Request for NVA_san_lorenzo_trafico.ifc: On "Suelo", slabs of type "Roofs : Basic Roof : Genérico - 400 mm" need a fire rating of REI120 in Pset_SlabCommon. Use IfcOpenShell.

First a look at what the model holds.

```python
import ifcopenshell
import ifcopenshell.util.element

model = ifcopenshell.open("NVA_san_lorenzo_trafico.ifc")
print(model.schema)
storey = next(s for s in model.by_type("IfcBuildingStorey") if s.Name == "Suelo")
slabs = [e for e in ifcopenshell.util.element.get_decomposition(storey) if e.is_a("IfcSlab")]
seen = {}
for e in slabs:
    element_type = ifcopenshell.util.element.get_type(e)
    key = (element_type.Name if element_type != e and element_type else None, ifcopenshell.util.element.get_pset(e, "Pset_SlabCommon", "FireRating"))
    seen[key] = seen.get(key, 0) + 1
for (name, value), count in sorted(seen.items(), key=str):
    print(count, "x", name, "|", value)
```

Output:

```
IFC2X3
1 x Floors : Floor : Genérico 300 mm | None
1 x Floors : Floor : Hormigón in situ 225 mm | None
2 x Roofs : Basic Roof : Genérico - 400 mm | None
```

```python
import ifcopenshell
import ifcopenshell.api.pset
import ifcopenshell.util.element

model = ifcopenshell.open("NVA_san_lorenzo_trafico.ifc")

storey = next(s for s in model.by_type("IfcBuildingStorey") if s.Name == "Suelo")
slabs = [e for e in ifcopenshell.util.element.get_decomposition(storey) if e.is_a("IfcSlab")]

count = 0
for e in slabs:
    element_type = ifcopenshell.util.element.get_type(e)
    if element_type in (None, e) or element_type.Name != "Roofs : Basic Roof : Genérico - 400 mm":
        continue
    # add_pset returns the element's existing set when there is one.
    pset = ifcopenshell.api.pset.add_pset(model, product=e, name="Pset_SlabCommon")
    ifcopenshell.api.pset.edit_pset(model, pset=pset, properties={"FireRating": "REI120"})
    count += 1

print(count, "slabs updated")

model.write("NVA_san_lorenzo_trafico_edited.ifc")
```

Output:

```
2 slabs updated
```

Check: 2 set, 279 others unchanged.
